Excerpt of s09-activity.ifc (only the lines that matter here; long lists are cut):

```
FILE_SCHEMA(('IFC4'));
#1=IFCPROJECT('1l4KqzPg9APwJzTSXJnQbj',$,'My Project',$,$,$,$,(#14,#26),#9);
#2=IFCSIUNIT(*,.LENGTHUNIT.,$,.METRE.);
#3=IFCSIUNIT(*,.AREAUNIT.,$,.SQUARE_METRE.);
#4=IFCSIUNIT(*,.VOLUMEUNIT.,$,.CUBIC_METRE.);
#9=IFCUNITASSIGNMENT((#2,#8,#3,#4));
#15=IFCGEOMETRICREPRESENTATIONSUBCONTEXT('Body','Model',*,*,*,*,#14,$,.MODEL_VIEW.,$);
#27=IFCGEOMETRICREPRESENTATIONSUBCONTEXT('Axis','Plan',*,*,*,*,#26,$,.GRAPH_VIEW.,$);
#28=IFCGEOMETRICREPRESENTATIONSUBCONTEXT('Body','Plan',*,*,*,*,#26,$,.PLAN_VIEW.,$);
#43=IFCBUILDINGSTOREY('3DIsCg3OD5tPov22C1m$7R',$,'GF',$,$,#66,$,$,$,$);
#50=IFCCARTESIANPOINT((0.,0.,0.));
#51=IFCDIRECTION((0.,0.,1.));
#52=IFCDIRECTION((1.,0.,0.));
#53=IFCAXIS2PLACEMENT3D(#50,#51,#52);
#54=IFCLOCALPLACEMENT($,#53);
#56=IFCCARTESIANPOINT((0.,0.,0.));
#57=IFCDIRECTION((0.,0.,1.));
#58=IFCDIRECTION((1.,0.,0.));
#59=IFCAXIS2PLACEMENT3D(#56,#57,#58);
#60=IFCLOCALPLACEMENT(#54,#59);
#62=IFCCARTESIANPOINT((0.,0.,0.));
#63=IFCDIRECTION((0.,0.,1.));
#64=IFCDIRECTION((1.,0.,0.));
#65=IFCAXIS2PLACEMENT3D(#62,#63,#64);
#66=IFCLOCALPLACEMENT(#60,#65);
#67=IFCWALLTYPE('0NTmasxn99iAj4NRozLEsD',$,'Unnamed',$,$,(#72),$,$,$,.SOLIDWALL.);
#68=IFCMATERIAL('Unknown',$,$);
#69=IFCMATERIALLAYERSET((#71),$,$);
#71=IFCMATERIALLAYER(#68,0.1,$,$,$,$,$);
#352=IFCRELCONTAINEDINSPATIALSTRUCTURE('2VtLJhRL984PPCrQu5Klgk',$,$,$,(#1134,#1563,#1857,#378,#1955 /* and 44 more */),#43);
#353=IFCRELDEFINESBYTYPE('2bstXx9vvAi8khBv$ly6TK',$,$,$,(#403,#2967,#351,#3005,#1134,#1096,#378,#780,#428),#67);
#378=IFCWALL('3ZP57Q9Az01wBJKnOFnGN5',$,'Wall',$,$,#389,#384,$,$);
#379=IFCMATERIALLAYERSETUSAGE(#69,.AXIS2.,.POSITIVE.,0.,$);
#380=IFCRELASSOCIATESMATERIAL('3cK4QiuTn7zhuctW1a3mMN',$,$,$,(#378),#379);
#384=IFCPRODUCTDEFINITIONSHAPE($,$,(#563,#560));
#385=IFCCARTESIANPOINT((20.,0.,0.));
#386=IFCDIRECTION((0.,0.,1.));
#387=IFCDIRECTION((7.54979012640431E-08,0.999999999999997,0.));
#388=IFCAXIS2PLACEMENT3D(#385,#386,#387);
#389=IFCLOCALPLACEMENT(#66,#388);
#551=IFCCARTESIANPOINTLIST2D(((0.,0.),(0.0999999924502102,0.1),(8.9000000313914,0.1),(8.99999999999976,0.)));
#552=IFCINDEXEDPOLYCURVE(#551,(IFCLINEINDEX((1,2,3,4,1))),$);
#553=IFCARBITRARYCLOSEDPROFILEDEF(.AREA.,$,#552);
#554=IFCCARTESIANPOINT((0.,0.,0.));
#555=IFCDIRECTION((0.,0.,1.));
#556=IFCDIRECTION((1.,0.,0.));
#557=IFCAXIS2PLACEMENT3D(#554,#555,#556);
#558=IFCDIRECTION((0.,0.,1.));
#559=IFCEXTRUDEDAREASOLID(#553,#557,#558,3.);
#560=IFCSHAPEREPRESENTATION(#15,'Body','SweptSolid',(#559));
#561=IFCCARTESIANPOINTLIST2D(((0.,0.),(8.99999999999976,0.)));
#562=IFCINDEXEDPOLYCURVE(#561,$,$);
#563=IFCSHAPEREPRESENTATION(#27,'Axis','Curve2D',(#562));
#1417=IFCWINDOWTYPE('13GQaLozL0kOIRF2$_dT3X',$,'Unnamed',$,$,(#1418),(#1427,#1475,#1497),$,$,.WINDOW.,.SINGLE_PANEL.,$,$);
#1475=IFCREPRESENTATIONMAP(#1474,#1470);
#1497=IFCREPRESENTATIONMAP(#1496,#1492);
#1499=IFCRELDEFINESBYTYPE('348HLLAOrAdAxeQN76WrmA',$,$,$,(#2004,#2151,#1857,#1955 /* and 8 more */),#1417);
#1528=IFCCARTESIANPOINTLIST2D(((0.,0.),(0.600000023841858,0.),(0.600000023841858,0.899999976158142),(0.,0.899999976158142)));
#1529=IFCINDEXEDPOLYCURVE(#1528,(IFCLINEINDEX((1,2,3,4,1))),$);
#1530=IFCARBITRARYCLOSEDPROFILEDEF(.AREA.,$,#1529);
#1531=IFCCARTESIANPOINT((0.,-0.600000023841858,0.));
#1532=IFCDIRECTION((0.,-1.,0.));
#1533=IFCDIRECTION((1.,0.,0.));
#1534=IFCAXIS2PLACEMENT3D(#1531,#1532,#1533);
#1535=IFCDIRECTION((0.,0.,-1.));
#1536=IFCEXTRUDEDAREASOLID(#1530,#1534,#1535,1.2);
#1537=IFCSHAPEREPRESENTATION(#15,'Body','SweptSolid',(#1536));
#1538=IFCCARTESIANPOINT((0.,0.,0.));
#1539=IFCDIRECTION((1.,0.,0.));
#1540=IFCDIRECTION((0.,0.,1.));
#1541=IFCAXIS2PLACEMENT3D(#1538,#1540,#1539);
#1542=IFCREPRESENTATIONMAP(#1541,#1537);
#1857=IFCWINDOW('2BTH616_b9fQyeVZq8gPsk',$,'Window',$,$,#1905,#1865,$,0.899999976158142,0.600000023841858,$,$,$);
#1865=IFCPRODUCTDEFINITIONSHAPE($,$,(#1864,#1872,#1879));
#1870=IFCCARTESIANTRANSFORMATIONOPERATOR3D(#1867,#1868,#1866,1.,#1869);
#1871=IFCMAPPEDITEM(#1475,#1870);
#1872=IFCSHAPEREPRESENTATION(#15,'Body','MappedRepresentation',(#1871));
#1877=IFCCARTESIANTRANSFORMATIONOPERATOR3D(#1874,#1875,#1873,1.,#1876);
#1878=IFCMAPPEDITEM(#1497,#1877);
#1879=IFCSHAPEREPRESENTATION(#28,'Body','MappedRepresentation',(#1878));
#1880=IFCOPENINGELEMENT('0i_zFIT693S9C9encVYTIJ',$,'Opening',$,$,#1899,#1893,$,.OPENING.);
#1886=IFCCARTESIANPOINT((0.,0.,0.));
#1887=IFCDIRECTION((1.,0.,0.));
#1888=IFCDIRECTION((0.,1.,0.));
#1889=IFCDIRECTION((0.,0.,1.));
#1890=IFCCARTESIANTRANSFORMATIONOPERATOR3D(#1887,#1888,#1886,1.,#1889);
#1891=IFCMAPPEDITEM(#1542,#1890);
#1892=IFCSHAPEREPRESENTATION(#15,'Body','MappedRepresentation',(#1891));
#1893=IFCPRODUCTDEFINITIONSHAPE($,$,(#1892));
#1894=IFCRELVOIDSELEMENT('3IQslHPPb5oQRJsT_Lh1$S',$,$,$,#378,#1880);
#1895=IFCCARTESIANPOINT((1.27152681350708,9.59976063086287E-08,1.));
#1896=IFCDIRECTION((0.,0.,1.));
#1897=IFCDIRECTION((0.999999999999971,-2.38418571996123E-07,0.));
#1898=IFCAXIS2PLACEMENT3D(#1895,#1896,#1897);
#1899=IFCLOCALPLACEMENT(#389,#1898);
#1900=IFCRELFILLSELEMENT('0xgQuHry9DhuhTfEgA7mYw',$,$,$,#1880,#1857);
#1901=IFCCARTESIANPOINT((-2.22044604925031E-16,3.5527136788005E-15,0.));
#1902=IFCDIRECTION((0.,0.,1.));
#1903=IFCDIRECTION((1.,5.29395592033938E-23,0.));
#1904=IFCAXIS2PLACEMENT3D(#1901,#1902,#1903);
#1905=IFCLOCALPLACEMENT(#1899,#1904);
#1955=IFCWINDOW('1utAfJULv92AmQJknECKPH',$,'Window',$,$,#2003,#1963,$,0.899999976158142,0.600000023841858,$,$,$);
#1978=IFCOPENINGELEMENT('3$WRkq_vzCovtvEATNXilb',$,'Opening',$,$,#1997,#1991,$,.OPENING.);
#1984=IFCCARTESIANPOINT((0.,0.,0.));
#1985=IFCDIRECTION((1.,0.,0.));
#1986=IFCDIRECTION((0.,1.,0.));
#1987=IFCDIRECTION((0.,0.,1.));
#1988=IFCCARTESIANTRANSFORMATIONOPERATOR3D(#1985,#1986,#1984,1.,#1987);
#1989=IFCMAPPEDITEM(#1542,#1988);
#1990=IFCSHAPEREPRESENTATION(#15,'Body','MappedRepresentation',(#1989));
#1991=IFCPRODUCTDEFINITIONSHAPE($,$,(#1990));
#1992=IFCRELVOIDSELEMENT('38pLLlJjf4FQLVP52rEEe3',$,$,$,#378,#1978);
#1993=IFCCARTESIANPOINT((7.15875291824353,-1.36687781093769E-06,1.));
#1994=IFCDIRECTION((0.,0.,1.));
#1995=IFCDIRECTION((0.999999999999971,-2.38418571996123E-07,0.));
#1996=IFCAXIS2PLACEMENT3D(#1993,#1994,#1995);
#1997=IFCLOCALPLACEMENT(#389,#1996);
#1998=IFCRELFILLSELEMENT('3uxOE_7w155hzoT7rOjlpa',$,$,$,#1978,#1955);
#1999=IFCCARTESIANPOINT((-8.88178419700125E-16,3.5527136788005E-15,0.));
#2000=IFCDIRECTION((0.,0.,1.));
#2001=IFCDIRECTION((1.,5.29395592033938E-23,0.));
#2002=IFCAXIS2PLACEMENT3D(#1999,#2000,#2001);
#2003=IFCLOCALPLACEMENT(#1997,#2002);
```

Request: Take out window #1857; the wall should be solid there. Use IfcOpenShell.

```python
import ifcopenshell
import ifcopenshell.api.feature
import ifcopenshell.api.root
import ifcopenshell.geom
import ifcopenshell.util.shape

model = ifcopenshell.open("s09-activity.ifc")
settings = ifcopenshell.geom.settings()


def volume(element):
    """Net volume in cubic metres, openings subtracted."""
    shape = ifcopenshell.geom.create_shape(settings, element)
    return ifcopenshell.util.shape.get_volume(shape.geometry)


window = model.by_guid("2BTH616_b9fQyeVZq8gPsk")
opening = window.FillsVoids[0].RelatingOpeningElement
wall = opening.VoidsElements[0].RelatingBuildingElement
before = volume(wall)

ifcopenshell.api.root.remove_product(model, product=window)
ifcopenshell.api.feature.remove_feature(model, feature=opening)

after = volume(wall)

print(f"wall volume {before:.3f} -> {after:.3f} m3")

model.write("s09-activity_v2.ifc")
```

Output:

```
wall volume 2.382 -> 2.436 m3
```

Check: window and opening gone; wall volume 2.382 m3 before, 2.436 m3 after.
